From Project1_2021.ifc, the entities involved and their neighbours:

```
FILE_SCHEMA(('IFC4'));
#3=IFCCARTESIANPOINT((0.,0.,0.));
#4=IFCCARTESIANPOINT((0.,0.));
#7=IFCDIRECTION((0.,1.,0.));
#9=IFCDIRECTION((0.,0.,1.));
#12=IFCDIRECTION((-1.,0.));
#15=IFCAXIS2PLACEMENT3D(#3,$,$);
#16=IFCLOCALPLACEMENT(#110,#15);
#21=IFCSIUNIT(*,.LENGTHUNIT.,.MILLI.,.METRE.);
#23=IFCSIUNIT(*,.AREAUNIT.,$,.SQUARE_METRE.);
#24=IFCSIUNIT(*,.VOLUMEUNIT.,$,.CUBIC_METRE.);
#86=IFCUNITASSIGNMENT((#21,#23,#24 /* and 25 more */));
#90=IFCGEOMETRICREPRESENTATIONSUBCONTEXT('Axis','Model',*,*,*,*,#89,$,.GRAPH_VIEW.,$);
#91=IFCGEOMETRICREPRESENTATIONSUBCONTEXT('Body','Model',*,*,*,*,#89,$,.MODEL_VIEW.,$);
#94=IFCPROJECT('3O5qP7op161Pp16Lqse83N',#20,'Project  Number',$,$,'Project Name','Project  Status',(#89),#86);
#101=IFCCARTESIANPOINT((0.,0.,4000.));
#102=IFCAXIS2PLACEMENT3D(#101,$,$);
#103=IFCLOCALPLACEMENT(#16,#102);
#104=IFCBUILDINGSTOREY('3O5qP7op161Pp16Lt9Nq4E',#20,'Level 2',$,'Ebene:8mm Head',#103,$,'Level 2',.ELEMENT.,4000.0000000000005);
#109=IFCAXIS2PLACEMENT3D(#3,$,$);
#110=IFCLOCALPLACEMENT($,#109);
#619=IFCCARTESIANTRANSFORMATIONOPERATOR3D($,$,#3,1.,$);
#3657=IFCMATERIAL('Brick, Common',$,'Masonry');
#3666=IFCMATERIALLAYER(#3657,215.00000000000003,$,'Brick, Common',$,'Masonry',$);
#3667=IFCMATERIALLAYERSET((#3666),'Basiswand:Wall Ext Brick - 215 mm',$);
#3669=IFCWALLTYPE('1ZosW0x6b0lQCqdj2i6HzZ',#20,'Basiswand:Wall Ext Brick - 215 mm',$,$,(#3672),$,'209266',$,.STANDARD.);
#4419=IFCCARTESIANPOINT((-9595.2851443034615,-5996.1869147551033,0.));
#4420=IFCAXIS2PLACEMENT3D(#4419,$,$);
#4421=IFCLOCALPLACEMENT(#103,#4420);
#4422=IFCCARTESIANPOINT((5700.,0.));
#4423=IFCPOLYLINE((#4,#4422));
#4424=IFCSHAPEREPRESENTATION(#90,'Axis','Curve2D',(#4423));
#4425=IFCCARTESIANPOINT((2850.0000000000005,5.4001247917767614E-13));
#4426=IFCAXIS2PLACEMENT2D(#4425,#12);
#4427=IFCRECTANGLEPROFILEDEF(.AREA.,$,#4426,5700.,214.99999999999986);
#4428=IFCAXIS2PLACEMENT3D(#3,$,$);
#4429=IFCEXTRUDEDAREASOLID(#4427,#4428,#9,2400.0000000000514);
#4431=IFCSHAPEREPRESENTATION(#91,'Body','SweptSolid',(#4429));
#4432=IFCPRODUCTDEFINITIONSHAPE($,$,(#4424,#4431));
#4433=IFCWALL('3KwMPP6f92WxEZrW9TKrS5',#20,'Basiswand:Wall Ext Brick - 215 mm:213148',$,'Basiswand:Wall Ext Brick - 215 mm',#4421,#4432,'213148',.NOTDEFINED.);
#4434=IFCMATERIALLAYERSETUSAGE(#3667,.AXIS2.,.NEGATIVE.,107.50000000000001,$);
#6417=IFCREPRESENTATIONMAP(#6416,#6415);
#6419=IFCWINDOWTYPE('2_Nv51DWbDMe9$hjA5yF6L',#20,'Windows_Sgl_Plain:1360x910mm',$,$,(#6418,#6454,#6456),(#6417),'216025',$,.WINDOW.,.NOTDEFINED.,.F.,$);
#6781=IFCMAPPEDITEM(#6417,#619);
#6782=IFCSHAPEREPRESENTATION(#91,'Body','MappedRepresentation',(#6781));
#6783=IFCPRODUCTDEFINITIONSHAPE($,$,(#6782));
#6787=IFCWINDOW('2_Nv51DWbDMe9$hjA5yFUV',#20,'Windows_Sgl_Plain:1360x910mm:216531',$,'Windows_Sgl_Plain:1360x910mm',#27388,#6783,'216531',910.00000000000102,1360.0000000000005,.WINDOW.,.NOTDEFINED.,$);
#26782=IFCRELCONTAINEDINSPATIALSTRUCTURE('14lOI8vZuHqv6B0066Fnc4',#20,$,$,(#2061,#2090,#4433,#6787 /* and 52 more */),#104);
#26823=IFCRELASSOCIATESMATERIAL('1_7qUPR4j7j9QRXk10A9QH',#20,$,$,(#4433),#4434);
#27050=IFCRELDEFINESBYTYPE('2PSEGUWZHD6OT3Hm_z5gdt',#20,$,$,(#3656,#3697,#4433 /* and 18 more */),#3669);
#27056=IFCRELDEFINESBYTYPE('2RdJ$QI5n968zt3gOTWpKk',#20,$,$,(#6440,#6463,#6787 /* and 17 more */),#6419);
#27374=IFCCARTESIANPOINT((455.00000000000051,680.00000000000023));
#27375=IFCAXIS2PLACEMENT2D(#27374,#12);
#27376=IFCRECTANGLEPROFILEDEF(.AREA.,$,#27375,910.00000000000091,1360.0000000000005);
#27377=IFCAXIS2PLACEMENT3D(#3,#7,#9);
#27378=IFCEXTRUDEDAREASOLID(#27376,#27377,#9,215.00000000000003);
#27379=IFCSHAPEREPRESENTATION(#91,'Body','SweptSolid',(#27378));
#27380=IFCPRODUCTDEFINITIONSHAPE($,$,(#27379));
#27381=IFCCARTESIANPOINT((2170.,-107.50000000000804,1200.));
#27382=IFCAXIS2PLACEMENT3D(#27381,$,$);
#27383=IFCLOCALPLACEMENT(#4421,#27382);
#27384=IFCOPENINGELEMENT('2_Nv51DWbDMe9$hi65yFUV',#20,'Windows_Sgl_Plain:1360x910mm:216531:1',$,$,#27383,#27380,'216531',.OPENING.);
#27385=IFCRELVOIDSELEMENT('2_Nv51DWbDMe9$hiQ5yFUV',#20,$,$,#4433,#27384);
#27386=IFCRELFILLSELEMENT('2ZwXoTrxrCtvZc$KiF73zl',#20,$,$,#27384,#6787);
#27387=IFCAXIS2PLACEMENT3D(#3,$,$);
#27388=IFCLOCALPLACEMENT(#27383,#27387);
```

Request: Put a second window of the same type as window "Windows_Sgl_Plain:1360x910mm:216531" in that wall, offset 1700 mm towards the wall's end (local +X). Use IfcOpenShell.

```python
import ifcopenshell
import ifcopenshell.api.feature
import ifcopenshell.api.geometry
import ifcopenshell.api.root
import ifcopenshell.geom
import ifcopenshell.util.element
import ifcopenshell.util.placement
import ifcopenshell.util.shape

model = ifcopenshell.open("Project1_2021.ifc")
settings = ifcopenshell.geom.settings()


def volume(element):
    """Net volume in cubic metres, openings subtracted."""
    shape = ifcopenshell.geom.create_shape(settings, element)
    return ifcopenshell.util.shape.get_volume(shape.geometry)


def reuse_history(source, copy):
    """copy_class also copies each property set's owner history, people and application; keep the originals."""
    for rel in copy.IsDefinedBy:
        if rel.is_a("IfcRelDefinesByProperties") and (history := rel.RelatingPropertyDefinition.OwnerHistory):
            rel.RelatingPropertyDefinition.OwnerHistory = source.OwnerHistory
            ifcopenshell.util.element.remove_deep2(model, history)


window = model.by_guid("2_Nv51DWbDMe9$hjA5yFUV")
opening = window.FillsVoids[0].RelatingOpeningElement
wall = opening.VoidsElements[0].RelatingBuildingElement
before = volume(wall)
shift = ifcopenshell.util.placement.get_local_placement(wall.ObjectPlacement)[:3, 0] * 1700.0

# copy_class copies the void relationship, type, container and properties, but no geometry.
new_opening = ifcopenshell.api.root.copy_class(model, product=opening)
new_opening.Representation = ifcopenshell.util.element.copy_deep(
    model, opening.Representation, exclude=["IfcGeometricRepresentationContext", "IfcRepresentationMap"]
)
new_opening.Name = "Windows_Sgl_Plain:1360x910mm"
new_opening.Tag = None
new_window = ifcopenshell.api.root.copy_class(model, product=window)
new_window.Representation = ifcopenshell.util.element.copy_deep(
    model, window.Representation, exclude=["IfcGeometricRepresentationContext", "IfcRepresentationMap"]
)
new_window.Name = "Windows_Sgl_Plain:1360x910mm"
new_window.Tag = None
reuse_history(window, new_window)
ifcopenshell.api.feature.add_filling(model, opening=new_opening, element=new_window)

for old, new in ((opening, new_opening), (window, new_window)):
    matrix = ifcopenshell.util.placement.get_local_placement(old.ObjectPlacement)
    matrix[:3, 3] += shift
    ifcopenshell.api.geometry.edit_object_placement(model, product=new, matrix=matrix, is_si=False)

after = volume(wall)

print(f"wall volume {before:.3f} -> {after:.3f} m3")

model.write("Project1_2021-out.ifc")
```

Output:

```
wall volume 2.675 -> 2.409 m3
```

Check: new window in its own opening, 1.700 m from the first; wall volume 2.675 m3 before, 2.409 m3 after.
